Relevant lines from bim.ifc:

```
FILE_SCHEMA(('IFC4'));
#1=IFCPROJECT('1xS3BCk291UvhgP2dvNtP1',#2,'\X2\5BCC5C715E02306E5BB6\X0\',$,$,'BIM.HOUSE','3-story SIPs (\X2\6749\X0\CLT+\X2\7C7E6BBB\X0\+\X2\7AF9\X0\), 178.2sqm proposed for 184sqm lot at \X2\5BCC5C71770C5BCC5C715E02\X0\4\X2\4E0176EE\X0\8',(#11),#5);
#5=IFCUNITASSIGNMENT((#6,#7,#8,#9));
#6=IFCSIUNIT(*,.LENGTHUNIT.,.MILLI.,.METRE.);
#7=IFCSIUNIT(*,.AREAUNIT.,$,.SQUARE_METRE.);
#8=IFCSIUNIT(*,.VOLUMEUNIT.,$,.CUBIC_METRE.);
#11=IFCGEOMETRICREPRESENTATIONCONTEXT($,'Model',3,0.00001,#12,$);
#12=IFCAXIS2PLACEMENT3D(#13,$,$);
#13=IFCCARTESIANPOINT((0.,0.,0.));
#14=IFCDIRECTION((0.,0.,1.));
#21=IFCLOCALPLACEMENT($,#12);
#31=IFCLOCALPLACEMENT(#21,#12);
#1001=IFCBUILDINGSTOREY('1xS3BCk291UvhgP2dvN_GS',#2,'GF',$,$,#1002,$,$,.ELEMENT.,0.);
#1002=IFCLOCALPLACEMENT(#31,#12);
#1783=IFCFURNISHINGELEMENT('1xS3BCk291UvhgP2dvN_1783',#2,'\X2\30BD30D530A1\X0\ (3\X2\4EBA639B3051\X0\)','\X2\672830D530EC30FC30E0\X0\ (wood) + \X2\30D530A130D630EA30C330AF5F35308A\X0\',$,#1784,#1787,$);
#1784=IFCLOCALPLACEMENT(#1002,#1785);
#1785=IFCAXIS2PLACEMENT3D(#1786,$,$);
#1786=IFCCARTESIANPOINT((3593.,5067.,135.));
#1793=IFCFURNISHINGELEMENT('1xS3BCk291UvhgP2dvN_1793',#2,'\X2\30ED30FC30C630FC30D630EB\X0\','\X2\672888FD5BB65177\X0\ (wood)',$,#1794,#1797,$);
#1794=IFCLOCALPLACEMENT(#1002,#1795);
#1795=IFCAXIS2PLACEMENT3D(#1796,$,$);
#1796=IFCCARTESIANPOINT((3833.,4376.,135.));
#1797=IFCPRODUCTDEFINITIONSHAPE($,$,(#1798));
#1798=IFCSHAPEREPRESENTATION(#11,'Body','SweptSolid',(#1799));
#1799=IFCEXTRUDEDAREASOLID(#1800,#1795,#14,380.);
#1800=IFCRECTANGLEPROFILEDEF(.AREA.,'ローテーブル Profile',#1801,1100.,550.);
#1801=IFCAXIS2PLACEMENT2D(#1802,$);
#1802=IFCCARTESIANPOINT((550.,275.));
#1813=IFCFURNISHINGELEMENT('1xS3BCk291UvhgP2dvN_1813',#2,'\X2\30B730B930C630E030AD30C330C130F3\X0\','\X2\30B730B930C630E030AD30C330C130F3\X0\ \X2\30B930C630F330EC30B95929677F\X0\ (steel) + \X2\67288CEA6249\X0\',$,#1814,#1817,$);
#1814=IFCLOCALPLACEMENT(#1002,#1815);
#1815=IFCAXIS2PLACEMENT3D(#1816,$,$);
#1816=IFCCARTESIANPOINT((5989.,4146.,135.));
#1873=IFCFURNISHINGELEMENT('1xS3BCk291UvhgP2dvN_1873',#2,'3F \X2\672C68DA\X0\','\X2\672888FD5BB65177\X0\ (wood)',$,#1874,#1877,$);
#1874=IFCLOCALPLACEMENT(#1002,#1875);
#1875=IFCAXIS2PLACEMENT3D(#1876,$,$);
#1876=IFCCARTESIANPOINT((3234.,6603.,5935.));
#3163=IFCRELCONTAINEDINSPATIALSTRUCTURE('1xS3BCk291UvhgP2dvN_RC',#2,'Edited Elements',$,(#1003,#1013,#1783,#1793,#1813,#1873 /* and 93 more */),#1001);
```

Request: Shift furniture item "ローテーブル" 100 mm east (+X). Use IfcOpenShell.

```python
import ifcopenshell
import ifcopenshell.api.geometry
import ifcopenshell.util.placement

model = ifcopenshell.open("bim.ifc")

item = model.by_id(1793)
matrix = ifcopenshell.util.placement.get_local_placement(item.ObjectPlacement)
matrix[0, 3] += 100.0
ifcopenshell.api.geometry.edit_object_placement(model, product=item, matrix=matrix, is_si=False)

print(ifcopenshell.util.placement.get_local_placement(item.ObjectPlacement).round(3) + 0.0)

model.write("bim_edited.ifc")
```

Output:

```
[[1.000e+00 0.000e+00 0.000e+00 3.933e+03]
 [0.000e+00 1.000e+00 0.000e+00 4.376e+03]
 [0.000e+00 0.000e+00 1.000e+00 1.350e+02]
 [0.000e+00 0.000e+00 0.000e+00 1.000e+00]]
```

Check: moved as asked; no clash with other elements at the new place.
